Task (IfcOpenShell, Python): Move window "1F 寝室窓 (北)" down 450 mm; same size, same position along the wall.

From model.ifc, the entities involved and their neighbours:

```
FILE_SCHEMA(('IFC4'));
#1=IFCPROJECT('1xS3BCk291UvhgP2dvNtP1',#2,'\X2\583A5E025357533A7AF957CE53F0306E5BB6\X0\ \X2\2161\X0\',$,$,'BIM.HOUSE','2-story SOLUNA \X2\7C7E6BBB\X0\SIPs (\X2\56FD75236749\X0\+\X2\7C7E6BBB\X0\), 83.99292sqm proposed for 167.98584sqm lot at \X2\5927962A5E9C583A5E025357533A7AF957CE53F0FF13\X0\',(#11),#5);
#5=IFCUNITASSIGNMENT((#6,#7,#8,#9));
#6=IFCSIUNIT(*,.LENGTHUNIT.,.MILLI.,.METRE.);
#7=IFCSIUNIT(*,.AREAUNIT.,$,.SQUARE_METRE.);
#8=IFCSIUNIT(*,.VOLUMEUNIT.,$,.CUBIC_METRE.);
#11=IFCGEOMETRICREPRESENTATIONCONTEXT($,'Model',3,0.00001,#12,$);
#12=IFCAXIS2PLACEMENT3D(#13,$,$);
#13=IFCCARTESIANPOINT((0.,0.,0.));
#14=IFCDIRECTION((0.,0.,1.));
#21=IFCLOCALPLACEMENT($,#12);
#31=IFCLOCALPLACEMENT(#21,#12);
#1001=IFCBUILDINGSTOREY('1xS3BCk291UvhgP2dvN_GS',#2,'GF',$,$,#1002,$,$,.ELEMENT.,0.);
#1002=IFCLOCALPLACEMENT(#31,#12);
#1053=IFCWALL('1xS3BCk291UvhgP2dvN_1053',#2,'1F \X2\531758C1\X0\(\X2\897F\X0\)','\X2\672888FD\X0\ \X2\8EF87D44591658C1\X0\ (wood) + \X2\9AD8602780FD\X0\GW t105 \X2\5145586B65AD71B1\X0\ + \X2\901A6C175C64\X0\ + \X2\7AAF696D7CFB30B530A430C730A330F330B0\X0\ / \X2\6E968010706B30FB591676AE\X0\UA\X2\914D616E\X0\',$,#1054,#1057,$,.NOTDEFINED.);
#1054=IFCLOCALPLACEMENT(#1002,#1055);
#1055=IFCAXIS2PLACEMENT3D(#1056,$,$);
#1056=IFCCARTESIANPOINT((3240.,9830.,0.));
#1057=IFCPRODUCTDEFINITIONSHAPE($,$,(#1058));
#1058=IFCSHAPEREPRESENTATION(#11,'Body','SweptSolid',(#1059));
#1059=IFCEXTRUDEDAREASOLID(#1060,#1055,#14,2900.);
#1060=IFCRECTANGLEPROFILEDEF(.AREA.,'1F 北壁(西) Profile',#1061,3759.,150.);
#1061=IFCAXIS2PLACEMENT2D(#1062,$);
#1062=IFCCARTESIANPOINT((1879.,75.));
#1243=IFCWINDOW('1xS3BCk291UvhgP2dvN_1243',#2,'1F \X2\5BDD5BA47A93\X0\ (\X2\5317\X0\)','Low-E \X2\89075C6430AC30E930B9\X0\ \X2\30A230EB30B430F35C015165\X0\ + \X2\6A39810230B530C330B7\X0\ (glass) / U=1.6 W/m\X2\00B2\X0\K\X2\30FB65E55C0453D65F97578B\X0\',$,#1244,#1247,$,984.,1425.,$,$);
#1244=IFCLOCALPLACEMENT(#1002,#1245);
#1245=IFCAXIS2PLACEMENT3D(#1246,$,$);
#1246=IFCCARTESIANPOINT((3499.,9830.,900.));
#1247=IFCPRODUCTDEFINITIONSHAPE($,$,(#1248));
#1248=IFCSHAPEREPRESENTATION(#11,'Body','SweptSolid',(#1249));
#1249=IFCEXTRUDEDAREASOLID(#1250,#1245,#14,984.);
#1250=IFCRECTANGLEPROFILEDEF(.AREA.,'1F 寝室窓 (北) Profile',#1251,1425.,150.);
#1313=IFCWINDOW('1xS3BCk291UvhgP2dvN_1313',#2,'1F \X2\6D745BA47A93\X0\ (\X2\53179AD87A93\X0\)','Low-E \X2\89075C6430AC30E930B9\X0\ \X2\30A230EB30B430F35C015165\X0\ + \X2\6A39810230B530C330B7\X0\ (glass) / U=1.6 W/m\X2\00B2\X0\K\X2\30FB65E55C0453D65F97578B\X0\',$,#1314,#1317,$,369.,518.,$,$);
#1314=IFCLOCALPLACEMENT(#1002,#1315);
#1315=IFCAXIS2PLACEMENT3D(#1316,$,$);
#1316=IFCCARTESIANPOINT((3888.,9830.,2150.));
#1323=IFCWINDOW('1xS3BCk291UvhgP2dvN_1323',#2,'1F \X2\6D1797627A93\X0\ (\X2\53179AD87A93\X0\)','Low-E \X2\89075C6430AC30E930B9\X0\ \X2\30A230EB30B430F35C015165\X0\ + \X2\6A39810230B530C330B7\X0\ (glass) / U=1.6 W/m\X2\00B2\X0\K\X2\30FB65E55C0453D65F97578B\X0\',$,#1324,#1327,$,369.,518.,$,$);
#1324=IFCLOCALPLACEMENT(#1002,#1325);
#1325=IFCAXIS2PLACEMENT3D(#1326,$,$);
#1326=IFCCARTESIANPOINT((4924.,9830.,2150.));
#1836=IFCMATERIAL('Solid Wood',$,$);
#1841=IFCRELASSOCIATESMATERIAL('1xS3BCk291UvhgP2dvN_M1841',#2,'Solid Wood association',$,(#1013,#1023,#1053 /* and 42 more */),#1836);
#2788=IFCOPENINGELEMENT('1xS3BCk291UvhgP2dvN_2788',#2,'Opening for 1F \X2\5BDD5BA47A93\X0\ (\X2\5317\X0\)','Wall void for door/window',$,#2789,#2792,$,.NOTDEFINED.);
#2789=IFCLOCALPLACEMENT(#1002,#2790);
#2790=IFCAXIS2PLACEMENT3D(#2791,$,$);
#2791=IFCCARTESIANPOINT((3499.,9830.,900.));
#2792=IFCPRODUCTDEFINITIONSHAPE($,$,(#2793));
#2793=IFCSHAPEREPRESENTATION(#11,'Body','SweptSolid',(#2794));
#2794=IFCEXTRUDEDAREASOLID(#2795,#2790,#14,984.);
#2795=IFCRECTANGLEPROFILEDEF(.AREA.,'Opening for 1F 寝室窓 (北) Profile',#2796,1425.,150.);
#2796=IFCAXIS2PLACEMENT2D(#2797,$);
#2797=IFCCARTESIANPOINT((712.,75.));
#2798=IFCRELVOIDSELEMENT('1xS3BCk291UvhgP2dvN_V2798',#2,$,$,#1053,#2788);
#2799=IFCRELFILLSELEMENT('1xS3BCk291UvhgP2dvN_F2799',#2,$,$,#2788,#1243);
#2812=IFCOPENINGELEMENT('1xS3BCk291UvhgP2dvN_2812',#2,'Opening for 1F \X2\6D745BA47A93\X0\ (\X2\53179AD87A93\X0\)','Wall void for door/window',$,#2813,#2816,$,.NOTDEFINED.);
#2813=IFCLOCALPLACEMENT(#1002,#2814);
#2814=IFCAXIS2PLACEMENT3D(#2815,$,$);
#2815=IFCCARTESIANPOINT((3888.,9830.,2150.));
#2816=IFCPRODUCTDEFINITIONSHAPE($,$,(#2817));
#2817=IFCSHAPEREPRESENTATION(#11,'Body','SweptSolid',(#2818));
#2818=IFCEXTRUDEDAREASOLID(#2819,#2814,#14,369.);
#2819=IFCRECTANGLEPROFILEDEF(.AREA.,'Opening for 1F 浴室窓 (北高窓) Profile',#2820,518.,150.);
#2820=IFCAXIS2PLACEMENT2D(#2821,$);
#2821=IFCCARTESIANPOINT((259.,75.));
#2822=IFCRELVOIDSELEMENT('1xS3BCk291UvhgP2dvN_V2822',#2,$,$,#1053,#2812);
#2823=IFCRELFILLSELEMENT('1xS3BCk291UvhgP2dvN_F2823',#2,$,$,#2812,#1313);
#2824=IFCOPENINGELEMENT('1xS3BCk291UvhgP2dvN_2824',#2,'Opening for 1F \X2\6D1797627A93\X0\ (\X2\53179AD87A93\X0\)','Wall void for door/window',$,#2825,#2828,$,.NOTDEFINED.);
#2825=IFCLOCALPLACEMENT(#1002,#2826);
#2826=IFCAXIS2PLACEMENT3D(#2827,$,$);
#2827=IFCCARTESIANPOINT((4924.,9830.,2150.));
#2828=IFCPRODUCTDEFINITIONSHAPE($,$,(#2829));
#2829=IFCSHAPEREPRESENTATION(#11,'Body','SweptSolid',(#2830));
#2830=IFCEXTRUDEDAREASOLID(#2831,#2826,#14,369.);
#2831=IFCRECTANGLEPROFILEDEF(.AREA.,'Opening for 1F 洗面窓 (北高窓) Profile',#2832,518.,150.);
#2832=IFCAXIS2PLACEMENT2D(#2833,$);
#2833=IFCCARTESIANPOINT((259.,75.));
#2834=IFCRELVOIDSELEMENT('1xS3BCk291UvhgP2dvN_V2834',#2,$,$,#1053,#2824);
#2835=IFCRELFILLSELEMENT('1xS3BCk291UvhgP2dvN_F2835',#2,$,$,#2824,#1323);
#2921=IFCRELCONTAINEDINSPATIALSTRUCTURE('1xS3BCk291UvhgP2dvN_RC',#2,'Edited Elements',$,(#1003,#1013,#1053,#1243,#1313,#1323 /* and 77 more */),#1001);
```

```python
import numpy as np
import ifcopenshell
import ifcopenshell.api.geometry
import ifcopenshell.util.placement
import ifcopenshell.util.unit

model = ifcopenshell.open("model.ifc")
unit_scale = ifcopenshell.util.unit.calculate_unit_scale(model)

window = model.by_id(1243)
opening = window.FillsVoids[0].RelatingOpeningElement
dz = -0.45 / unit_scale

shift = np.array([0.0, 0.0, dz])
# The window is not placed relative to its opening, so move both.
for product in (opening, window):
    matrix = ifcopenshell.util.placement.get_local_placement(product.ObjectPlacement)
    matrix[:3, 3] += shift
    ifcopenshell.api.geometry.edit_object_placement(model, product=product, matrix=matrix, is_si=False)

print(f"moved by {dz * unit_scale:+.3f} m")

model.write("model_updated.ifc")
```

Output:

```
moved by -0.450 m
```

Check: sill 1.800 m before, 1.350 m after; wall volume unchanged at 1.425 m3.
